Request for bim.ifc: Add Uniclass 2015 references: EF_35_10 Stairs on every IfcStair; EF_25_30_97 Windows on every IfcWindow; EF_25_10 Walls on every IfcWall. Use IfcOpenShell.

First a look at what the model holds.

```python
import ifcopenshell

model = ifcopenshell.open("bim.ifc")
print(model.schema)
print("classifications:", [c.Name for c in model.by_type("IfcClassification")])
for ifc_class in ("IfcDoor", "IfcRoof", "IfcStair", "IfcWall", "IfcWindow"):
    print(ifc_class, len(model.by_type(ifc_class)))
```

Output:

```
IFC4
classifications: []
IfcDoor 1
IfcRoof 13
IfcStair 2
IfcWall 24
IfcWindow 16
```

```python
import ifcopenshell
import ifcopenshell.api.classification

model = ifcopenshell.open("bim.ifc")

system = ifcopenshell.api.classification.add_classification(model, classification="Uniclass 2015")

codes = {
    "IfcStair": ("EF_35_10", "Stairs"),
    "IfcWindow": ("EF_25_30_97", "Windows"),
    "IfcWall": ("EF_25_10", "Walls"),
}
for ifc_class, (code, name) in codes.items():
    products = model.by_type(ifc_class)
    ifcopenshell.api.classification.add_reference(
        model, products=products, classification=system, identification=code, name=name
    )
    print(code, len(products))

model.write("bim_v2.ifc")
```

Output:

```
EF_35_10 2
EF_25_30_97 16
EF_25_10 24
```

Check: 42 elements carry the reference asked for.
